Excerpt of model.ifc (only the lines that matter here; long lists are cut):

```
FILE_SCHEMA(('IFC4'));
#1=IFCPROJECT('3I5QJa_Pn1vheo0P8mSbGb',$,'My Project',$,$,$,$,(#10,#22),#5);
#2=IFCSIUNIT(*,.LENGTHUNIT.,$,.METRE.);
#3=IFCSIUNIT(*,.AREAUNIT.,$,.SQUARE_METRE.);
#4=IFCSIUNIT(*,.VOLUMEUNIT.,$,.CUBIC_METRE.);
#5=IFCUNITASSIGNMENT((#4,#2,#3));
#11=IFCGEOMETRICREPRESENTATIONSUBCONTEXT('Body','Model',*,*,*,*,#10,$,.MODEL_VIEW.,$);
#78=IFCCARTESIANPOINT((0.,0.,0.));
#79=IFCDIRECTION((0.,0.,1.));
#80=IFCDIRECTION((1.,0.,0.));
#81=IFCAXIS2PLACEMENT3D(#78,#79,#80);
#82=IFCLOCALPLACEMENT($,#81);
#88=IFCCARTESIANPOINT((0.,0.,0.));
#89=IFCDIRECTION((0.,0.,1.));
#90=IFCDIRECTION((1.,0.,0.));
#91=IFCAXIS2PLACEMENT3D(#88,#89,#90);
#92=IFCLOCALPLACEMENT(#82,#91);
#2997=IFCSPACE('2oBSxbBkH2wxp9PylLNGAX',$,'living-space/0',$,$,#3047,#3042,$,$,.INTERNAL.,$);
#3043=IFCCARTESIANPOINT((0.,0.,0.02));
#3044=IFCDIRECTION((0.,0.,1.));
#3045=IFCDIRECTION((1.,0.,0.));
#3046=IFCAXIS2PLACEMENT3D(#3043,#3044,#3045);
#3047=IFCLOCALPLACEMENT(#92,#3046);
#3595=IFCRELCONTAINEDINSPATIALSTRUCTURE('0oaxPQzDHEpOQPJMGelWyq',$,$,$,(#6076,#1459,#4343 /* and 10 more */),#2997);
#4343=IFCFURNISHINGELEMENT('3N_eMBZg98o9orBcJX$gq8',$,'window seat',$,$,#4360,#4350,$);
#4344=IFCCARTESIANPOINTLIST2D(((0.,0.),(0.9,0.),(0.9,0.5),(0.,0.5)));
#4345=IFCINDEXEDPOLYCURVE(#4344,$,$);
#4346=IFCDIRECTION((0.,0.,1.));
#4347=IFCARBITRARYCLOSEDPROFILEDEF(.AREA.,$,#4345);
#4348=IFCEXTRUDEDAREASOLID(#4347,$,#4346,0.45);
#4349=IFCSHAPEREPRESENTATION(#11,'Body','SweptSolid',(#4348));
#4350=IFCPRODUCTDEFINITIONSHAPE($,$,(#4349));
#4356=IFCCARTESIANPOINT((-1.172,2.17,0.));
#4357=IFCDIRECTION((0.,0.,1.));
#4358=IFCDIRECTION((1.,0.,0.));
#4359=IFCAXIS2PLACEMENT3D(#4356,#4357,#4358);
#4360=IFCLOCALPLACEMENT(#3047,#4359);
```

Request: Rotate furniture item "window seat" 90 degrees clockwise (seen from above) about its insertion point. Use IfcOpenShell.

```python
import ifcopenshell
import ifcopenshell.api.geometry
import ifcopenshell.util.placement

model = ifcopenshell.open("model.ifc")

item = model.by_guid("3N_eMBZg98o9orBcJX$gq8")
matrix = ifcopenshell.util.placement.get_local_placement(item.ObjectPlacement)
matrix = matrix @ ifcopenshell.util.placement.rotation(-90, "Z")
ifcopenshell.api.geometry.edit_object_placement(model, product=item, matrix=matrix, is_si=False)

print(ifcopenshell.util.placement.get_local_placement(item.ObjectPlacement).round(3) + 0.0)

model.write("model_rev.ifc")
```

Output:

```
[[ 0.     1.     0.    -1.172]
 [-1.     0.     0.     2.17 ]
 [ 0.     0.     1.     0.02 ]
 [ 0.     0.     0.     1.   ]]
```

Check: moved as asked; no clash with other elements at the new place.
